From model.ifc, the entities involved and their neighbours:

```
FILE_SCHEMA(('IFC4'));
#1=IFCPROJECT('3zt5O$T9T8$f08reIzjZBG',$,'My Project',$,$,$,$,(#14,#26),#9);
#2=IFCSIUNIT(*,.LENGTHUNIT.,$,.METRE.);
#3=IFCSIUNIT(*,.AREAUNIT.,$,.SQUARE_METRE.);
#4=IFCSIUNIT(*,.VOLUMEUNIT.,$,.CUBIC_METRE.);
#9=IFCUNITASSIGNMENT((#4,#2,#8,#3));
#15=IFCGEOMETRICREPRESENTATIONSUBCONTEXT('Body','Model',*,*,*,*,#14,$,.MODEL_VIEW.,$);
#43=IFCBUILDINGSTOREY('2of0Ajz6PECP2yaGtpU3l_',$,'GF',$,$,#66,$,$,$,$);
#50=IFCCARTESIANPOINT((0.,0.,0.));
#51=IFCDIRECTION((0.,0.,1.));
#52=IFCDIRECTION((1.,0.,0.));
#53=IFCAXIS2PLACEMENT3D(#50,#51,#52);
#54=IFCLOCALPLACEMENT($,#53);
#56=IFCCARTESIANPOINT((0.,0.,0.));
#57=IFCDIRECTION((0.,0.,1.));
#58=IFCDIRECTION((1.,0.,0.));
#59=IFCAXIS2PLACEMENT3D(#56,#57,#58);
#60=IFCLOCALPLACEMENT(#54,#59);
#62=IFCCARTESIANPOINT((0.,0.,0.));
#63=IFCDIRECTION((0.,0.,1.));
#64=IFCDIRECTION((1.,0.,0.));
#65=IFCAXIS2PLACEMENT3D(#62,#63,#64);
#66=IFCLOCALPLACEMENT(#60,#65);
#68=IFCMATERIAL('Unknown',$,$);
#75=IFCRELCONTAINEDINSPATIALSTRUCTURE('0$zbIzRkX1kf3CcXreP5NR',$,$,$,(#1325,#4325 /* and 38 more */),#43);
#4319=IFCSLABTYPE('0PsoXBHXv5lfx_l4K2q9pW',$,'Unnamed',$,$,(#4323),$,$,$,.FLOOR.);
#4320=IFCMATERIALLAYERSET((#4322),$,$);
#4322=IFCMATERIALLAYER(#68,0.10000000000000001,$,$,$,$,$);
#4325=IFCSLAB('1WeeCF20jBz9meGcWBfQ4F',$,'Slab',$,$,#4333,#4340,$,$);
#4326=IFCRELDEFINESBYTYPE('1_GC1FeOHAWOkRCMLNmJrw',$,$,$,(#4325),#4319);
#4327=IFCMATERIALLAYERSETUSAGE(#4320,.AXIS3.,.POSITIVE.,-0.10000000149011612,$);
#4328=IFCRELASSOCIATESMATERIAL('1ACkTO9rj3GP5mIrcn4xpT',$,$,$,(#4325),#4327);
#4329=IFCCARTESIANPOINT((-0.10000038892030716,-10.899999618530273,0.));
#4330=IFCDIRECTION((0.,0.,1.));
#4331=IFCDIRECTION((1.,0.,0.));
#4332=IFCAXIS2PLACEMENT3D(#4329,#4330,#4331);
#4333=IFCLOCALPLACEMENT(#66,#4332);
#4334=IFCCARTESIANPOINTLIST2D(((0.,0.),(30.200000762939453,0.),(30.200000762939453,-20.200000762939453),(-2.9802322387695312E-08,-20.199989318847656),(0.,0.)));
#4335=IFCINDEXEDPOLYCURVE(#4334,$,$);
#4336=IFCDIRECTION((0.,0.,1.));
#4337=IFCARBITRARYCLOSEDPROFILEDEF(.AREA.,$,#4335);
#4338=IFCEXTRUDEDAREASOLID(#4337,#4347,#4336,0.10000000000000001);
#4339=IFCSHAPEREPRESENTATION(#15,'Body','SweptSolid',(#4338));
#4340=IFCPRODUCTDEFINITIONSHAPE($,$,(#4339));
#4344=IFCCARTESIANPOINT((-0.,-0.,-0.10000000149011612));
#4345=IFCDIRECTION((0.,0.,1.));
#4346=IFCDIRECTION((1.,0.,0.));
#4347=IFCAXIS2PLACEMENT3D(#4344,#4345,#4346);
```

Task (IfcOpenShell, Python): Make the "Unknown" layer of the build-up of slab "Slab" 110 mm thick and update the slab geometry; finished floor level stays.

```python
import ifcopenshell
import ifcopenshell.util.element
import ifcopenshell.util.representation
import ifcopenshell.util.unit

model = ifcopenshell.open("model.ifc")
unit_scale = ifcopenshell.util.unit.calculate_unit_scale(model)

layer_set = model.by_id(4320)
layer = next(l for l in layer_set.MaterialLayers if l.Material and l.Material.Name == "Unknown")
change = 0.11 / unit_scale - layer.LayerThickness
layer.LayerThickness += change

# Geometry does not follow the layer set by itself.
slabs = [e for e in ifcopenshell.util.element.get_elements_by_material(model, layer_set) if e.is_a("IfcSlab")]
for slab in sorted(slabs, key=lambda e: e.id()):
    body = ifcopenshell.util.representation.get_representation(slab, "Model", "Body")
    solid = body.Items[0]
    old_depth = solid.Depth
    solid.Depth += change
    # Extruded upwards: lower the start of the extrusion so the top stays.
    x, y, z = solid.Position.Location.Coordinates
    solid.Position.Location = model.createIfcCartesianPoint((x, y, z - change))
    print(slab.id(), f"{old_depth:g} -> {solid.Depth:g}")

# The layers are counted up from the underside, which has moved.
for usage in {ifcopenshell.util.element.get_material(slab) for slab in slabs}:
    usage.OffsetFromReferenceLine -= change

model.write("model_v2.ifc")
```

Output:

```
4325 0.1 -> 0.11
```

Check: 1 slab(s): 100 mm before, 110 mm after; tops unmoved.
